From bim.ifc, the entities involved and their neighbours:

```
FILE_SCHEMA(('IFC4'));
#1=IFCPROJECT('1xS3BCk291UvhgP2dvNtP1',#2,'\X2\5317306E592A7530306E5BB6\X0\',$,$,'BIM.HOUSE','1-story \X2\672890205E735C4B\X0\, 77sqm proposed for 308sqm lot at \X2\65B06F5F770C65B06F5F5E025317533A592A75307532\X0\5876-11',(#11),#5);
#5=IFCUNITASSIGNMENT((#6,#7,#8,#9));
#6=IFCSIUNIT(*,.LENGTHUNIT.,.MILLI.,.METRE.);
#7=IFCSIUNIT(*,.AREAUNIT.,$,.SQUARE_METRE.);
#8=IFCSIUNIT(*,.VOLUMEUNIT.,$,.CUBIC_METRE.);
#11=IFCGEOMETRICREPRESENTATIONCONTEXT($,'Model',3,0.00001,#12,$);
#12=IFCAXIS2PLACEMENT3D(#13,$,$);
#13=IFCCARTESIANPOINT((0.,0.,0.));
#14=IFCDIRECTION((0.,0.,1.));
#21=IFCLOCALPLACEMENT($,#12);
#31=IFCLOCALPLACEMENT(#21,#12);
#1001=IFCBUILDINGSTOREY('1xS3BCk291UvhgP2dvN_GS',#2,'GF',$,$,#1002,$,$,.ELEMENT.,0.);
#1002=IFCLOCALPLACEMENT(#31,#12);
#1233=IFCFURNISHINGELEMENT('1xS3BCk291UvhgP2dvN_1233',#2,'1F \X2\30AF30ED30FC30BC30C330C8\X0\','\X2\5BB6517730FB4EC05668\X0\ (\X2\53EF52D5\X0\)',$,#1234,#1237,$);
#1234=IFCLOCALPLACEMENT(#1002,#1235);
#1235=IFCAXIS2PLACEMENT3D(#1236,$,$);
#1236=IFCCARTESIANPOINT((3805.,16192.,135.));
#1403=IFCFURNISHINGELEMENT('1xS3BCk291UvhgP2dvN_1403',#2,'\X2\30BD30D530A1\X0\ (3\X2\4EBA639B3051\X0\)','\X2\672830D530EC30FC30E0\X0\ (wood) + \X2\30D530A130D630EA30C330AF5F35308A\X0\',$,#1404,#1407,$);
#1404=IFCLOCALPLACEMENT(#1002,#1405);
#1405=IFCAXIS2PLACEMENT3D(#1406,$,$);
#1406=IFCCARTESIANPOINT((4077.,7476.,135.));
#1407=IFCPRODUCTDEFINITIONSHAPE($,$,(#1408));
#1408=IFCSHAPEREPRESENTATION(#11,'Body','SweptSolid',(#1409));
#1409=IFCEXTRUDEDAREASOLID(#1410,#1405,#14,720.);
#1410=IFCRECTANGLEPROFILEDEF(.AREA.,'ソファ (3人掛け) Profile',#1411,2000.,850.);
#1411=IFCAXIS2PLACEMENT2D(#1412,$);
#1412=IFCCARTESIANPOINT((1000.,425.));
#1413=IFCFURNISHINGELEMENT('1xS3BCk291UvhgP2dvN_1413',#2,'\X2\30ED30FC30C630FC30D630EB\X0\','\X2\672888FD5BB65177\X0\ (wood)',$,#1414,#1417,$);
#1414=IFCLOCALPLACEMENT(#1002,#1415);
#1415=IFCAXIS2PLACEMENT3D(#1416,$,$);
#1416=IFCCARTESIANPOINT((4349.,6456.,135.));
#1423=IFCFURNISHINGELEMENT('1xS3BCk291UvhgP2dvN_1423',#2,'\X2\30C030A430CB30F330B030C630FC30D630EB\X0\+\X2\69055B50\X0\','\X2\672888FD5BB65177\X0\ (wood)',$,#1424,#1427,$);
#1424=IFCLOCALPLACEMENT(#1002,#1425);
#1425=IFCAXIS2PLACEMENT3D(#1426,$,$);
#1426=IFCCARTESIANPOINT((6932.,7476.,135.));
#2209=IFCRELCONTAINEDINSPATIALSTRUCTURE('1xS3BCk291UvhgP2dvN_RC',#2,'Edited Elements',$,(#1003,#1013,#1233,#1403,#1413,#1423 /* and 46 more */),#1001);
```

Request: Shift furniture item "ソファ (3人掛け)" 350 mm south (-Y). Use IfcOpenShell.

```python
import ifcopenshell
import ifcopenshell.api.geometry
import ifcopenshell.util.placement
import ifcopenshell.util.unit

model = ifcopenshell.open("bim.ifc")
unit_scale = ifcopenshell.util.unit.calculate_unit_scale(model)

item = model.by_id(1403)
matrix = ifcopenshell.util.placement.get_local_placement(item.ObjectPlacement)
matrix[1, 3] -= 0.35 / unit_scale
ifcopenshell.api.geometry.edit_object_placement(model, product=item, matrix=matrix, is_si=False)

print(ifcopenshell.util.placement.get_local_placement(item.ObjectPlacement).round(3) + 0.0)

model.write("bim_v2.ifc")
```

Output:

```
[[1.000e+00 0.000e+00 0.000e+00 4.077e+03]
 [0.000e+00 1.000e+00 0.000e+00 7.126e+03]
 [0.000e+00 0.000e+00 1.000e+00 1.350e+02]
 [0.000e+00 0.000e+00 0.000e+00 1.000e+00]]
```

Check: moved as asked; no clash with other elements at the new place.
